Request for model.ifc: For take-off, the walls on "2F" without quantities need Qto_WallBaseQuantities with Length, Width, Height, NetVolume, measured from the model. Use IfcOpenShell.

First a look at what the model holds.

```python
import ifcopenshell
import ifcopenshell.util.element
import ifcopenshell.util.unit

model = ifcopenshell.open("model.ifc")
print(model.schema)
for unit_type in ("LENGTHUNIT", "AREAUNIT", "VOLUMEUNIT"):
    print(unit_type, ifcopenshell.util.unit.calculate_unit_scale(model, unit_type))
storey = next(s for s in model.by_type("IfcBuildingStorey") if s.Name == "2F")
walls = [e for e in ifcopenshell.util.element.get_decomposition(storey) if e.is_a("IfcWall")]
for e in sorted(walls, key=lambda e: e.id()):
    print(e.id(), e.is_a(), e.Name, list(ifcopenshell.util.element.get_psets(e, qtos_only=True)), sep=" | ")
```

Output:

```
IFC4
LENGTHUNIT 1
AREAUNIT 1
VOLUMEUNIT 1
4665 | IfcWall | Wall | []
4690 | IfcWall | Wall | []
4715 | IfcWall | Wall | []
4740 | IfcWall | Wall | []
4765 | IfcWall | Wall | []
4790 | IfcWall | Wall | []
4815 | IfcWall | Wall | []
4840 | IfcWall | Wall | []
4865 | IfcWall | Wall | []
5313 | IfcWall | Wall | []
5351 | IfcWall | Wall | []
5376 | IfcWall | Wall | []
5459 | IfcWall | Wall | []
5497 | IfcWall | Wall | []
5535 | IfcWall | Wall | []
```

```python
import ifcopenshell
import ifcopenshell.api.pset
import ifcopenshell.geom
import ifcopenshell.util.element
import ifcopenshell.util.shape
import ifcopenshell.util.unit

model = ifcopenshell.open("model.ifc")
unit_scale = ifcopenshell.util.unit.calculate_unit_scale(model)
volume_scale = ifcopenshell.util.unit.calculate_unit_scale(model, "VOLUMEUNIT")
settings = ifcopenshell.geom.settings()

storey = next(s for s in model.by_type("IfcBuildingStorey") if s.Name == "2F")
walls = [e for e in ifcopenshell.util.element.get_decomposition(storey) if e.is_a("IfcWall")]

for e in sorted(walls, key=lambda e: e.id()):
    if ifcopenshell.util.element.get_psets(e, qtos_only=True, should_inherit=False):
        continue
    # Geometry comes back in metres, in the element's own axes.
    shape = ifcopenshell.geom.create_shape(settings, e)
    values = {
        "Length": ifcopenshell.util.shape.get_x(shape.geometry) / unit_scale,
        "Width": ifcopenshell.util.shape.get_y(shape.geometry) / unit_scale,
        "Height": ifcopenshell.util.shape.get_z(shape.geometry) / unit_scale,
        "NetVolume": ifcopenshell.util.shape.get_volume(shape.geometry) / volume_scale,
    }
    qto = ifcopenshell.api.pset.add_qto(model, product=e, name="Qto_WallBaseQuantities")
    ifcopenshell.api.pset.edit_qto(model, qto=qto, properties=values)
    print(e.id(), {k: round(v, 3) for k, v in values.items()})

model.write("model_updated.ifc")
```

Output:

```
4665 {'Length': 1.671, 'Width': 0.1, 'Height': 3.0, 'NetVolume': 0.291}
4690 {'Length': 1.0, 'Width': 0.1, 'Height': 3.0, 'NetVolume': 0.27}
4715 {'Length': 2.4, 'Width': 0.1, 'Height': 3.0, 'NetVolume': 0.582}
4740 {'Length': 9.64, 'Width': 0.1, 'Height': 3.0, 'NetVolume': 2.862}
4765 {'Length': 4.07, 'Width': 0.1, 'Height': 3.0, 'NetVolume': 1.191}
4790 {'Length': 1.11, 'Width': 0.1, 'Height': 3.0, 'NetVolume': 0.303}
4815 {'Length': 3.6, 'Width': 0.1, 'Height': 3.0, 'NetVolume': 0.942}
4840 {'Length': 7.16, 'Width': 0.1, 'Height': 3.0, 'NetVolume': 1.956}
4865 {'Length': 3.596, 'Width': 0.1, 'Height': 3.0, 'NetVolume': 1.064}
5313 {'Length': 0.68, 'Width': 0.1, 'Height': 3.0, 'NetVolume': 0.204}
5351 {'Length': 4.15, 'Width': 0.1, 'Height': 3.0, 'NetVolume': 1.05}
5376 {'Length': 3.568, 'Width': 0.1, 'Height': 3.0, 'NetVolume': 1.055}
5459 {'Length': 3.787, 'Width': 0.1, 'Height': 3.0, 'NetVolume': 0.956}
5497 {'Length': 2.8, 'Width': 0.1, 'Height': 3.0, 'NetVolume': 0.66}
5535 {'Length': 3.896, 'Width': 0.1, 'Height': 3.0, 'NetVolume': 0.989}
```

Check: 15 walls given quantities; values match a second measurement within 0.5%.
